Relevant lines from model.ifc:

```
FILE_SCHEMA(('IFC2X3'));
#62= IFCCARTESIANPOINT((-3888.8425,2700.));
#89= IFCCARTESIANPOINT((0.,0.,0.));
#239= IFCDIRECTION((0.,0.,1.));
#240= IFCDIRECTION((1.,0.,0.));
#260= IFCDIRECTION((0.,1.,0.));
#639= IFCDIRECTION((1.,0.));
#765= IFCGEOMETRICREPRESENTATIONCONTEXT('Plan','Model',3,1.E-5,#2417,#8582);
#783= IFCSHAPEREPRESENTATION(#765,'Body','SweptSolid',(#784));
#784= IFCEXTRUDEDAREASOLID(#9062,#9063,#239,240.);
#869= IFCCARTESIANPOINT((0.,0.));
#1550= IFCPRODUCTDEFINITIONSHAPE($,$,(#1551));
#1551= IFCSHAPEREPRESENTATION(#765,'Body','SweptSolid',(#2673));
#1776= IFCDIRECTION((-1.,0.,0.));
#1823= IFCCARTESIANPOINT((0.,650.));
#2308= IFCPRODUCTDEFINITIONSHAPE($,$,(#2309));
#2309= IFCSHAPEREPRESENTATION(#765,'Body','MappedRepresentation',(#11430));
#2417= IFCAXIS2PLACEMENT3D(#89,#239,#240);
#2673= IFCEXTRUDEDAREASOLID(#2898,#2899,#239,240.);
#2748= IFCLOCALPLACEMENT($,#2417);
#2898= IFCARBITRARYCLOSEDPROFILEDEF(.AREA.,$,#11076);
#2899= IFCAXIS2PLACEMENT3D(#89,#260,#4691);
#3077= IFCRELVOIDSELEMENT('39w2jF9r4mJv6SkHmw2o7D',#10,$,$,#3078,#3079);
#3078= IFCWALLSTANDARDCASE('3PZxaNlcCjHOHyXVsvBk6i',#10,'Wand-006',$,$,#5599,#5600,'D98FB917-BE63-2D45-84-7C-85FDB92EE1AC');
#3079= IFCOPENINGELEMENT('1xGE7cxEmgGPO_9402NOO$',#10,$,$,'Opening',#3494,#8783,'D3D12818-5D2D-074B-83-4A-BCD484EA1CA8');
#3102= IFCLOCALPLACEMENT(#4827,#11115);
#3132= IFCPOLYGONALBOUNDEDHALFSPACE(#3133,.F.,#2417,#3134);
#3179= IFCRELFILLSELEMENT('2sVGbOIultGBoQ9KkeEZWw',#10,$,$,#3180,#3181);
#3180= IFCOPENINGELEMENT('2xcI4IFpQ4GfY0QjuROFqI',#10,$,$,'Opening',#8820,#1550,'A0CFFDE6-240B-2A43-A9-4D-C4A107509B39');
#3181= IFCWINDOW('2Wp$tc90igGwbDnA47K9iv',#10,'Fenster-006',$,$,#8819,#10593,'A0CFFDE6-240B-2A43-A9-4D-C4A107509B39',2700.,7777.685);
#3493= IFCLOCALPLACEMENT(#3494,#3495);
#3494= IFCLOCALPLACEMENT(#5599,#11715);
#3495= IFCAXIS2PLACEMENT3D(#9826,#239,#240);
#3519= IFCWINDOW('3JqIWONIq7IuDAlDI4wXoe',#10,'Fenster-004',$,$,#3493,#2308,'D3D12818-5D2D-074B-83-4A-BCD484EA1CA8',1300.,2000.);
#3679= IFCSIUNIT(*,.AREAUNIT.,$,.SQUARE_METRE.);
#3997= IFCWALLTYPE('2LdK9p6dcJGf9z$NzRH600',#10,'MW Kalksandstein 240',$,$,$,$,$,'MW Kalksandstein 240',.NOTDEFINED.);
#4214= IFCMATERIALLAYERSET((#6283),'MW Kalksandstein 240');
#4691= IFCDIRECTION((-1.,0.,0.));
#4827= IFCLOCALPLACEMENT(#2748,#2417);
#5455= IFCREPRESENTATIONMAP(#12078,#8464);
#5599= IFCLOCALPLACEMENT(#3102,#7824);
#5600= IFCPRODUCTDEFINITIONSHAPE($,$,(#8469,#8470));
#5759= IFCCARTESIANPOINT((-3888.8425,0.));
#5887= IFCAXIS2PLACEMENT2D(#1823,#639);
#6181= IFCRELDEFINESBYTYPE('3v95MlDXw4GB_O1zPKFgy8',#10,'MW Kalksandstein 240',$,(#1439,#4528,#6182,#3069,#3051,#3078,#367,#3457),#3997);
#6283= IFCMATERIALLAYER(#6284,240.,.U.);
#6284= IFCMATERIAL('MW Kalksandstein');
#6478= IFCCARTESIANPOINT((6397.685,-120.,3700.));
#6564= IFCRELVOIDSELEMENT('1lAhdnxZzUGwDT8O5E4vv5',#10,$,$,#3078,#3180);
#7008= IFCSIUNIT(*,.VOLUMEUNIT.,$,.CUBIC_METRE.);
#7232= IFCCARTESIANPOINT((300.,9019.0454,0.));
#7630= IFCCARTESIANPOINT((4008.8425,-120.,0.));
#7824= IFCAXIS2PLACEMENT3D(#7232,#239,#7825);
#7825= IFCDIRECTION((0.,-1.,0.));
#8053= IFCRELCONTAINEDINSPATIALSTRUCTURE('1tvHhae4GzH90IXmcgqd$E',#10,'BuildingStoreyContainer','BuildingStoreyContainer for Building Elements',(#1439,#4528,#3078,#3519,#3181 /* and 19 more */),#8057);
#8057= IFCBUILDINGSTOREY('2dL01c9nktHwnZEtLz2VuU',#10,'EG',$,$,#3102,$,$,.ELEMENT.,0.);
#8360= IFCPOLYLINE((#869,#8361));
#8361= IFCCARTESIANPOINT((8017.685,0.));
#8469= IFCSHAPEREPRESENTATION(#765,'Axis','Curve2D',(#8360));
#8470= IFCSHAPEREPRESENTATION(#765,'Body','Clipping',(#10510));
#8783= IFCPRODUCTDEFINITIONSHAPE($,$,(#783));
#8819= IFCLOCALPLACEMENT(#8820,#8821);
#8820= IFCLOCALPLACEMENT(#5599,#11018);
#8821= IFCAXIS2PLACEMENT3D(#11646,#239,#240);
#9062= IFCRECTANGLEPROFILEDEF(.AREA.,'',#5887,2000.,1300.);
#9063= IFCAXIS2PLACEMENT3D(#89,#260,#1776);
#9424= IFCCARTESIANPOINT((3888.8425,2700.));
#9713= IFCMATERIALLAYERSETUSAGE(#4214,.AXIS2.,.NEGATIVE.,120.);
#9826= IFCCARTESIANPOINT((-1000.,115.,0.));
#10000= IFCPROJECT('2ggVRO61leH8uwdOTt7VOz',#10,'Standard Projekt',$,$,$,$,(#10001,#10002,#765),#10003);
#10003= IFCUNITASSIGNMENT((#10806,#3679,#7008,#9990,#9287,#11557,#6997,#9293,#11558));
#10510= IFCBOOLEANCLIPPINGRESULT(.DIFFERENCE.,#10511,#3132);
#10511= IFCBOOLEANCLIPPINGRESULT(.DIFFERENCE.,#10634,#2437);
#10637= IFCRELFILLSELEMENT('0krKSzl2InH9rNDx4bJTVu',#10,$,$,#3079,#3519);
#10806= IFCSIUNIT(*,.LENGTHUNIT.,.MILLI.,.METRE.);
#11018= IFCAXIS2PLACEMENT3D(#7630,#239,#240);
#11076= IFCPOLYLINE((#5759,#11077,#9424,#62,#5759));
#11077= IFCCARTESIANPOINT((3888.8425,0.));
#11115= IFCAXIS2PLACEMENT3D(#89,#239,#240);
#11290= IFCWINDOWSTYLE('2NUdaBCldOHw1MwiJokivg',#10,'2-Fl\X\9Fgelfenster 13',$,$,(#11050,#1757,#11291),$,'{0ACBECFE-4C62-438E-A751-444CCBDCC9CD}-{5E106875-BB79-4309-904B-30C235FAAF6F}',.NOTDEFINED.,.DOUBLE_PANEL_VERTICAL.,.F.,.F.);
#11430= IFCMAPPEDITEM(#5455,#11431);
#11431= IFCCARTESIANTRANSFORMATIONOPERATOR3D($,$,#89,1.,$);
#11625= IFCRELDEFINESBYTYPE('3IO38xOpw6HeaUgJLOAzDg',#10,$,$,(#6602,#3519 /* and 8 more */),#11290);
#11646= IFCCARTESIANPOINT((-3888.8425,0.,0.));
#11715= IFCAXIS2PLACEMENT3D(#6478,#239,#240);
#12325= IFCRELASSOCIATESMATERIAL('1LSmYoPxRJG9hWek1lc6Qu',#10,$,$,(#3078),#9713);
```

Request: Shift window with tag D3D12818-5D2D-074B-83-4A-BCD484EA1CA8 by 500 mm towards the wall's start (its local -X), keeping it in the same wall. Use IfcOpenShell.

```python
import ifcopenshell
import ifcopenshell.api.geometry
import ifcopenshell.util.placement
import ifcopenshell.util.unit

model = ifcopenshell.open("model.ifc")
unit_scale = ifcopenshell.util.unit.calculate_unit_scale(model)

window = model.by_id(3519)
opening = window.FillsVoids[0].RelatingOpeningElement
wall = opening.VoidsElements[0].RelatingBuildingElement

wall_matrix = ifcopenshell.util.placement.get_local_placement(wall.ObjectPlacement)
shift = wall_matrix[:3, 0] * -0.5 / unit_scale
before = ifcopenshell.util.placement.get_local_placement(window.ObjectPlacement)[:3, 3].copy()

# The window is placed relative to its opening, so it follows when the opening moves.
matrix = ifcopenshell.util.placement.get_local_placement(opening.ObjectPlacement)
matrix[:3, 3] += shift
ifcopenshell.api.geometry.edit_object_placement(
    model, product=opening, matrix=matrix, is_si=False, should_transform_children=True
)

after = ifcopenshell.util.placement.get_local_placement(window.ObjectPlacement)[:3, 3]
print("window moved by", (after - before).round(3) + 0.0)

model.write("model_v2.ifc")
```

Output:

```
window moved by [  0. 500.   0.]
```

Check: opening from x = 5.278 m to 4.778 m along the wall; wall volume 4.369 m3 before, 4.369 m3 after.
